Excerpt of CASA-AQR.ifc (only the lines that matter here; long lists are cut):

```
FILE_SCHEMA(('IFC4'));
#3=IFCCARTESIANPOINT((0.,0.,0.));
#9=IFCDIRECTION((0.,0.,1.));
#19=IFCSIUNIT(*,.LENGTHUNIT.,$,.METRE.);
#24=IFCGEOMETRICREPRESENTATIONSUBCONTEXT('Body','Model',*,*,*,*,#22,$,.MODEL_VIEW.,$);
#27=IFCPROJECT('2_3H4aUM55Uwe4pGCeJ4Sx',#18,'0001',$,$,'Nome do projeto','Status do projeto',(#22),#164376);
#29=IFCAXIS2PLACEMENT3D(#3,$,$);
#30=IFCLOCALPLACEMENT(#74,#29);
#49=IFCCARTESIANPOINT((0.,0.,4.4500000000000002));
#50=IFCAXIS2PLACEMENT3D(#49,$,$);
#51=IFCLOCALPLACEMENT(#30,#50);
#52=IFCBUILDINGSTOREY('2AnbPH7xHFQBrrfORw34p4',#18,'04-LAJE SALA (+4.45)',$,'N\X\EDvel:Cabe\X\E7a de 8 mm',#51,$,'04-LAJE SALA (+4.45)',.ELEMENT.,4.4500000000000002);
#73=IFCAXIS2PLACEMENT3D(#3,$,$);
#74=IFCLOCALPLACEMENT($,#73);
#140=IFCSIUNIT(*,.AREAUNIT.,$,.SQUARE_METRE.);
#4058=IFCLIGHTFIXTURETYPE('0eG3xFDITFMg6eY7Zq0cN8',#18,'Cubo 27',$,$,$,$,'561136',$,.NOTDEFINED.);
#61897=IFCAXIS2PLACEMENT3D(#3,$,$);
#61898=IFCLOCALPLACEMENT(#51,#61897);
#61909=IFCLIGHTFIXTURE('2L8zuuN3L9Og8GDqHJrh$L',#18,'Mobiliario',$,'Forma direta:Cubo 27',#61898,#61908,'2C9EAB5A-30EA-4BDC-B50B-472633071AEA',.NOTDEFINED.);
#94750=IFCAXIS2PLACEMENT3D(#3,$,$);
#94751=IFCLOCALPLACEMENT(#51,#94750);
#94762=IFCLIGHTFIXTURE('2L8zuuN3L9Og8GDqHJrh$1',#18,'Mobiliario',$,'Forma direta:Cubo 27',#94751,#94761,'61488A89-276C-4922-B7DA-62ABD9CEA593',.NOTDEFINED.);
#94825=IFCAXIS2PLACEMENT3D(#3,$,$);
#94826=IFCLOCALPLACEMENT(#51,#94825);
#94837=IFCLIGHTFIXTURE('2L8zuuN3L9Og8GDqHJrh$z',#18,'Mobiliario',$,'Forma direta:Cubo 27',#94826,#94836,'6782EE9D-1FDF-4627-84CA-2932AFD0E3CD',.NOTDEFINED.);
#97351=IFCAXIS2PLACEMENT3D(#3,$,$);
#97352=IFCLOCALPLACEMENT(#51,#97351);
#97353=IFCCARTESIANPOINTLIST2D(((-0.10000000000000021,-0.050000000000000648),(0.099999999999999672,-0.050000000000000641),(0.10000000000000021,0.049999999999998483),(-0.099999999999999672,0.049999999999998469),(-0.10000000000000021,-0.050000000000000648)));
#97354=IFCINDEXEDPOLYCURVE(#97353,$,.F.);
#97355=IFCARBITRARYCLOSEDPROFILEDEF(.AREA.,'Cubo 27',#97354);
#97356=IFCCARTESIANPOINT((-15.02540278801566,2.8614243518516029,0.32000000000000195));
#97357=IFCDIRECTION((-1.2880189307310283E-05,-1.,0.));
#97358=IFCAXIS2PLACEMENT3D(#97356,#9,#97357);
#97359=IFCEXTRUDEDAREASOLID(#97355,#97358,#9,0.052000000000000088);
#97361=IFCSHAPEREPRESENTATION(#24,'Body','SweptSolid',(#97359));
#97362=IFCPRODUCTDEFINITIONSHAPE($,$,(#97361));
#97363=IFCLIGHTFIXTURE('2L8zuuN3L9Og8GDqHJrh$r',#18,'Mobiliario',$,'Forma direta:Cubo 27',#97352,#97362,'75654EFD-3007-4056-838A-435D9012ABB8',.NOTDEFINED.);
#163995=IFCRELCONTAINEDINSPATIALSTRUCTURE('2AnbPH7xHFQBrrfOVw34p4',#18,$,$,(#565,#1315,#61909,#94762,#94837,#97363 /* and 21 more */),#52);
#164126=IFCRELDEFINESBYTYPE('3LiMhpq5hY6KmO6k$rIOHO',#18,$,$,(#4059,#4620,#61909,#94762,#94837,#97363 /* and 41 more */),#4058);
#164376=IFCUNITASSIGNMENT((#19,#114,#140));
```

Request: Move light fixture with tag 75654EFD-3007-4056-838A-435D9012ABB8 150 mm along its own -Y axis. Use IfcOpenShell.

```python
import ifcopenshell
import ifcopenshell.api.geometry
import ifcopenshell.util.placement
import ifcopenshell.util.unit

model = ifcopenshell.open("CASA-AQR.ifc")
unit_scale = ifcopenshell.util.unit.calculate_unit_scale(model)

item = model.by_guid("2L8zuuN3L9Og8GDqHJrh$r")
matrix = ifcopenshell.util.placement.get_local_placement(item.ObjectPlacement)
matrix[:3, 3] -= matrix[:3, 1] * 0.15 / unit_scale
ifcopenshell.api.geometry.edit_object_placement(model, product=item, matrix=matrix, is_si=False)

print(ifcopenshell.util.placement.get_local_placement(item.ObjectPlacement).round(3) + 0.0)

model.write("CASA-AQR_edited.ifc")
```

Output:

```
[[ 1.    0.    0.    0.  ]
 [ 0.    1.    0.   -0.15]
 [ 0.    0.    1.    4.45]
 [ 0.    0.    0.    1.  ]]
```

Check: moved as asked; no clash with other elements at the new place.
